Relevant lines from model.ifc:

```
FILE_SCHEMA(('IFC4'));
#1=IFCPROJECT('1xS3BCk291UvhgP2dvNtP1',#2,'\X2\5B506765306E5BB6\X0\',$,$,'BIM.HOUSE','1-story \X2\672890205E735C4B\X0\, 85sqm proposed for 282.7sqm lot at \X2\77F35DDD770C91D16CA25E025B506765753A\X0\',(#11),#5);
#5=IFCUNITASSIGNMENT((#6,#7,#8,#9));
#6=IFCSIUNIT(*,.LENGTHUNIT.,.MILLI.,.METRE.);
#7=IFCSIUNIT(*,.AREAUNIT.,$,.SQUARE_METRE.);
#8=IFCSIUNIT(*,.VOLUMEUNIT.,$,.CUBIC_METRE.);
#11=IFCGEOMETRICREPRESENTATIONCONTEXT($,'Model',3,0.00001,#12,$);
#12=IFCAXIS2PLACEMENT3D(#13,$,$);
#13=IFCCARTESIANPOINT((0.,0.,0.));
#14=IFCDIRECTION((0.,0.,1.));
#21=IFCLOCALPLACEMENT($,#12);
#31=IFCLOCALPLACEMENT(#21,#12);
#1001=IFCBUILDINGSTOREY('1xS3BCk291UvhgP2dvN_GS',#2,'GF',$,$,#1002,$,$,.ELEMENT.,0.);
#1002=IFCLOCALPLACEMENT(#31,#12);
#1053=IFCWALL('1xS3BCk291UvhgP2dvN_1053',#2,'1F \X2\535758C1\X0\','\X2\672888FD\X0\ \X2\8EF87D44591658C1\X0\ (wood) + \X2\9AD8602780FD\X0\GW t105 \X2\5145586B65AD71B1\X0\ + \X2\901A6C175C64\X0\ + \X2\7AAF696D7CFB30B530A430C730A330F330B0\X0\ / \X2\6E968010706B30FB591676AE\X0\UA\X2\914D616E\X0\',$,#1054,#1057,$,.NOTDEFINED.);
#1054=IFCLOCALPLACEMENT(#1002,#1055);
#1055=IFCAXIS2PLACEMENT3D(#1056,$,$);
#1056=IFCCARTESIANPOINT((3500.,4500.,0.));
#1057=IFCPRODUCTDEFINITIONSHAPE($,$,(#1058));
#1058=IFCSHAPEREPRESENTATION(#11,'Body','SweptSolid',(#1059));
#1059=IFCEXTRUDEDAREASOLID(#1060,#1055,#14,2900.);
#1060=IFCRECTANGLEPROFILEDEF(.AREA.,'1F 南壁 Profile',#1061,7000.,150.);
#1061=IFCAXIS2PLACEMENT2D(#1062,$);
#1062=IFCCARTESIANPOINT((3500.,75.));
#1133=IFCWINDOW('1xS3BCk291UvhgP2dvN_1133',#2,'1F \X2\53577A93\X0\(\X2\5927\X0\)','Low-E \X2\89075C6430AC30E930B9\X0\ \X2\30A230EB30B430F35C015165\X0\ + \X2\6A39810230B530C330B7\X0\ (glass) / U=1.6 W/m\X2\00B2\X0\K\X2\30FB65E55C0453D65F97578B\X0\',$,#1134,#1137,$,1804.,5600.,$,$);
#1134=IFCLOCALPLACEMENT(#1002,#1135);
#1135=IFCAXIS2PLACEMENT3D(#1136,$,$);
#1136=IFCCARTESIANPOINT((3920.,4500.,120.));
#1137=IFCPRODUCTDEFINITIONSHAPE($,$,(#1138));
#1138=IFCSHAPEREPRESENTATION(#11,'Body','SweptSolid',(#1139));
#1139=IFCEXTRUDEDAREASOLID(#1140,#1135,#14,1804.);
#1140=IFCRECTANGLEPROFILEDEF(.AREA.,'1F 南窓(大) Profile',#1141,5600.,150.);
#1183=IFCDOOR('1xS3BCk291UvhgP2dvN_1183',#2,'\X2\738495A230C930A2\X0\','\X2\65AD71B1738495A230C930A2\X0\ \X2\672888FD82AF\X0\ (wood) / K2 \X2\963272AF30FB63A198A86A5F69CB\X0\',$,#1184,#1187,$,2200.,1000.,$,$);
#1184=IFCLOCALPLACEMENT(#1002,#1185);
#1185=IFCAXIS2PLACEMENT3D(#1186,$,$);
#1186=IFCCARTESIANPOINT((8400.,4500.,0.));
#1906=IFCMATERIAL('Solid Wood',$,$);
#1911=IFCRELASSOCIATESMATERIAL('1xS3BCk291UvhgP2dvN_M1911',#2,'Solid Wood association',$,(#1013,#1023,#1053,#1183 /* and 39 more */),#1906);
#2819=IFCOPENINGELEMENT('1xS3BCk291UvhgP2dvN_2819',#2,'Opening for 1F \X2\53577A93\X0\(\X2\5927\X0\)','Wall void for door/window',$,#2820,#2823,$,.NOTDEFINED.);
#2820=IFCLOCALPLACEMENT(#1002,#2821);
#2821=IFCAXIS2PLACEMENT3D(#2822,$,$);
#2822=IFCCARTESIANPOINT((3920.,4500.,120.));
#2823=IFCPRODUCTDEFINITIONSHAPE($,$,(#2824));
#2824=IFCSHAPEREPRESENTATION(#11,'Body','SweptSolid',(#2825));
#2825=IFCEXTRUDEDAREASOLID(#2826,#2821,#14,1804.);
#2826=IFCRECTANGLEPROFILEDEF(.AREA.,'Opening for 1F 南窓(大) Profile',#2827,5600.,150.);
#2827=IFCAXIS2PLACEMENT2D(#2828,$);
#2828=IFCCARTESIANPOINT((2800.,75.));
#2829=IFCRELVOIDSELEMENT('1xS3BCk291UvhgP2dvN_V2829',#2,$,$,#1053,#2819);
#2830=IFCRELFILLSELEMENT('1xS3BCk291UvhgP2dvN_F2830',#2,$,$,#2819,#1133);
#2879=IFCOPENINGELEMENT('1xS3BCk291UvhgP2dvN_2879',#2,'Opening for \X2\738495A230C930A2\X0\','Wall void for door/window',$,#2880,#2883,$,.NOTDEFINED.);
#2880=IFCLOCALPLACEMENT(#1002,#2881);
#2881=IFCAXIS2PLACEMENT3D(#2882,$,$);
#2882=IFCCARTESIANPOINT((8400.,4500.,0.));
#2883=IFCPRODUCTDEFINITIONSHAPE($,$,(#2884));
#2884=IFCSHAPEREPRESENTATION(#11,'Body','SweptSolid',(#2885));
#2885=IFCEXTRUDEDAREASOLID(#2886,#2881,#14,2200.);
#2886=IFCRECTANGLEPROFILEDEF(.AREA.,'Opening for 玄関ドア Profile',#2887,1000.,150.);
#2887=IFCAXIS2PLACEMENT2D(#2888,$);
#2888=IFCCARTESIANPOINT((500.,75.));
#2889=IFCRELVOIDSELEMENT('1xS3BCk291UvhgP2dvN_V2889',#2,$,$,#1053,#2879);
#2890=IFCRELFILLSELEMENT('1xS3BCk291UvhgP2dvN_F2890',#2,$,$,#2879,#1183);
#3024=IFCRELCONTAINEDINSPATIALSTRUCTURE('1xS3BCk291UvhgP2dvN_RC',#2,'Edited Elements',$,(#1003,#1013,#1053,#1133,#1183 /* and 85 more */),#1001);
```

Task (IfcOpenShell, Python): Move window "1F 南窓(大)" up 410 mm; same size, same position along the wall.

```python
import numpy as np
import ifcopenshell
import ifcopenshell.api.geometry
import ifcopenshell.util.placement
import ifcopenshell.util.unit

model = ifcopenshell.open("model.ifc")
unit_scale = ifcopenshell.util.unit.calculate_unit_scale(model)

window = model.by_id(1133)
opening = window.FillsVoids[0].RelatingOpeningElement
dz = 0.41 / unit_scale

shift = np.array([0.0, 0.0, dz])
# The window is not placed relative to its opening, so move both.
for product in (opening, window):
    matrix = ifcopenshell.util.placement.get_local_placement(product.ObjectPlacement)
    matrix[:3, 3] += shift
    ifcopenshell.api.geometry.edit_object_placement(model, product=product, matrix=matrix, is_si=False)

print(f"moved by {dz * unit_scale:+.3f} m")

model.write("model_updated.ifc")
```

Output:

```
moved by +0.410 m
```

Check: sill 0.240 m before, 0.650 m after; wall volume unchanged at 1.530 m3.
